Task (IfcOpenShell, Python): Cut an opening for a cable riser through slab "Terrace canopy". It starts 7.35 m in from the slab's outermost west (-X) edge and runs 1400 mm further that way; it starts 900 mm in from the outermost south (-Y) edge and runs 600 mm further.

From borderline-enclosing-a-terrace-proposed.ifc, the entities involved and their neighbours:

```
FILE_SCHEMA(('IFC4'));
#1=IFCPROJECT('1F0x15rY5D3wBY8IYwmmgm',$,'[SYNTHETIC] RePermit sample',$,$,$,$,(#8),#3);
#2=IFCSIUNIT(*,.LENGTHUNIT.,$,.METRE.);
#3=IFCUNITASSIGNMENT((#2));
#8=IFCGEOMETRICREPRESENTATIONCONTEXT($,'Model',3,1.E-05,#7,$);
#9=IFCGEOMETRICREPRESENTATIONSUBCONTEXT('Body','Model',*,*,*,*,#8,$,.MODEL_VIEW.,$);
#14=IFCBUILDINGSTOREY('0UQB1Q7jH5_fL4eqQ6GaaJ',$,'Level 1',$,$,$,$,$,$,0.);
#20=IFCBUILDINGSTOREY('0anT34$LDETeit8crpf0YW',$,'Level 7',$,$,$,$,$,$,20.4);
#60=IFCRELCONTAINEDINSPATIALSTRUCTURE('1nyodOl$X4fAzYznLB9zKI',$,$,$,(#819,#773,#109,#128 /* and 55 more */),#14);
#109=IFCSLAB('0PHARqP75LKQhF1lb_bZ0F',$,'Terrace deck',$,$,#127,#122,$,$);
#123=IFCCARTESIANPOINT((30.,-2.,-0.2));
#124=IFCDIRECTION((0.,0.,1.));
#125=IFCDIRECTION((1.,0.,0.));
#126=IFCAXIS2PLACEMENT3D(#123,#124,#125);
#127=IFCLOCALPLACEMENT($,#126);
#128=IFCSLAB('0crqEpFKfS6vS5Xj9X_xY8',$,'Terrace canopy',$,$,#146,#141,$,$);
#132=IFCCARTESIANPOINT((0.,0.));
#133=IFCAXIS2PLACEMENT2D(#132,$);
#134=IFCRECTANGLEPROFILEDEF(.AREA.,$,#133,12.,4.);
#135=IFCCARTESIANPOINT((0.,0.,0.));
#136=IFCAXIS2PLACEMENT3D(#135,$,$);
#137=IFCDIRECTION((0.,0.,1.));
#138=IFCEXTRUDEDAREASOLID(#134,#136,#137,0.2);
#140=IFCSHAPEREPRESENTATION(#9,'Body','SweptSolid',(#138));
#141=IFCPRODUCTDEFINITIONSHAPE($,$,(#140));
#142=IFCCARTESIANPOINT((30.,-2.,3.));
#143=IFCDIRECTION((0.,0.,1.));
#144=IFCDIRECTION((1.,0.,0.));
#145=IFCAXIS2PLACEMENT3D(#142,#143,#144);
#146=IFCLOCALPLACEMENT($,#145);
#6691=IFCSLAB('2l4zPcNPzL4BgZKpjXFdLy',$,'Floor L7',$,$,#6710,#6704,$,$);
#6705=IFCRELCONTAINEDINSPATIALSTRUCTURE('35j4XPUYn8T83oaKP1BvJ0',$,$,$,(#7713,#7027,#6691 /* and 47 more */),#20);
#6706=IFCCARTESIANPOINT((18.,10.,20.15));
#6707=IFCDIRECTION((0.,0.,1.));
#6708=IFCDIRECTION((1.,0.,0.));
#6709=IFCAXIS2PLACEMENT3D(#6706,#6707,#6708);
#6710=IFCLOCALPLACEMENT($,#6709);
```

```python
import numpy as np
import ifcopenshell
import ifcopenshell.api.feature
import ifcopenshell.api.geometry
import ifcopenshell.api.root
import ifcopenshell.geom
import ifcopenshell.util.placement
import ifcopenshell.util.representation
import ifcopenshell.util.shape
import ifcopenshell.util.unit

model = ifcopenshell.open("borderline-enclosing-a-terrace-proposed.ifc")
unit_scale = ifcopenshell.util.unit.calculate_unit_scale(model)
settings = ifcopenshell.geom.settings()


def volume(element):
    """Net volume in cubic metres, openings subtracted."""
    shape = ifcopenshell.geom.create_shape(settings, element)
    return ifcopenshell.util.shape.get_volume(shape.geometry)


slab = model.by_guid("0crqEpFKfS6vS5Xj9X_xY8")
before = volume(slab)

# Extent in the slab's own axes, in metres. The edges named are its -X and -Y sides.
slab_shape = ifcopenshell.geom.create_shape(settings, slab)
vertices = ifcopenshell.util.shape.get_vertices(slab_shape.geometry)
x_min, y_min, bottom = vertices.min(axis=0)
top = vertices[:, 2].max()

opening = ifcopenshell.api.root.create_entity(model, ifc_class="IfcOpeningElement", name="Cable riser opening", predefined_type="OPENING")
context = ifcopenshell.util.representation.get_context(model, "Model", "Body", "MODEL_VIEW")
width, depth = 1.4, 0.6
outline = [(0.0, 0.0), (width, 0.0), (width, depth), (0.0, depth), (0.0, 0.0)]
# Overshoot both faces by 50 mm so the cut is clean.
shape = ifcopenshell.api.geometry.add_slab_representation(
    model, context=context, depth=top - bottom + 0.1, polyline=outline
)
ifcopenshell.api.geometry.assign_representation(model, product=opening, representation=shape)

matrix = ifcopenshell.util.placement.get_local_placement(slab.ObjectPlacement)
matrix[:, 3] = matrix @ np.append(np.array([x_min + 7.35, y_min + 0.9, bottom - 0.05]) / unit_scale, 1.0)
ifcopenshell.api.geometry.edit_object_placement(model, product=opening, matrix=matrix, is_si=False)
ifcopenshell.api.feature.add_feature(model, feature=opening, element=slab)

after = volume(slab)

print(f"slab volume {before:.3f} -> {after:.3f} m3")

model.write("borderline-enclosing-a-terrace-proposed_updated.ifc")
```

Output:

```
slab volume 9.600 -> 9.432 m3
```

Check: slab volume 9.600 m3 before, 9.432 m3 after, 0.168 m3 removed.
